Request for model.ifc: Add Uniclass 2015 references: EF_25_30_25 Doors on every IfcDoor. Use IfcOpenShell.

First a look at what the model holds.

```python
import ifcopenshell

model = ifcopenshell.open("model.ifc")
print(model.schema)
print("classifications:", [c.Name for c in model.by_type("IfcClassification")])
for ifc_class in ("IfcDoor", "IfcRoof", "IfcStair", "IfcWall", "IfcWindow"):
    print(ifc_class, len(model.by_type(ifc_class)))
```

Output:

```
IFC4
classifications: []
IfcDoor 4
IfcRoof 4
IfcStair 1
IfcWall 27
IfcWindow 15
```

```python
import ifcopenshell
import ifcopenshell.api.classification

model = ifcopenshell.open("model.ifc")

system = ifcopenshell.api.classification.add_classification(model, classification="Uniclass 2015")

codes = {
    "IfcDoor": ("EF_25_30_25", "Doors"),
}
for ifc_class, (code, name) in codes.items():
    products = model.by_type(ifc_class)
    ifcopenshell.api.classification.add_reference(
        model, products=products, classification=system, identification=code, name=name
    )
    print(code, len(products))

model.write("model_updated.ifc")
```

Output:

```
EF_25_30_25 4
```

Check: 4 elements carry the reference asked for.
